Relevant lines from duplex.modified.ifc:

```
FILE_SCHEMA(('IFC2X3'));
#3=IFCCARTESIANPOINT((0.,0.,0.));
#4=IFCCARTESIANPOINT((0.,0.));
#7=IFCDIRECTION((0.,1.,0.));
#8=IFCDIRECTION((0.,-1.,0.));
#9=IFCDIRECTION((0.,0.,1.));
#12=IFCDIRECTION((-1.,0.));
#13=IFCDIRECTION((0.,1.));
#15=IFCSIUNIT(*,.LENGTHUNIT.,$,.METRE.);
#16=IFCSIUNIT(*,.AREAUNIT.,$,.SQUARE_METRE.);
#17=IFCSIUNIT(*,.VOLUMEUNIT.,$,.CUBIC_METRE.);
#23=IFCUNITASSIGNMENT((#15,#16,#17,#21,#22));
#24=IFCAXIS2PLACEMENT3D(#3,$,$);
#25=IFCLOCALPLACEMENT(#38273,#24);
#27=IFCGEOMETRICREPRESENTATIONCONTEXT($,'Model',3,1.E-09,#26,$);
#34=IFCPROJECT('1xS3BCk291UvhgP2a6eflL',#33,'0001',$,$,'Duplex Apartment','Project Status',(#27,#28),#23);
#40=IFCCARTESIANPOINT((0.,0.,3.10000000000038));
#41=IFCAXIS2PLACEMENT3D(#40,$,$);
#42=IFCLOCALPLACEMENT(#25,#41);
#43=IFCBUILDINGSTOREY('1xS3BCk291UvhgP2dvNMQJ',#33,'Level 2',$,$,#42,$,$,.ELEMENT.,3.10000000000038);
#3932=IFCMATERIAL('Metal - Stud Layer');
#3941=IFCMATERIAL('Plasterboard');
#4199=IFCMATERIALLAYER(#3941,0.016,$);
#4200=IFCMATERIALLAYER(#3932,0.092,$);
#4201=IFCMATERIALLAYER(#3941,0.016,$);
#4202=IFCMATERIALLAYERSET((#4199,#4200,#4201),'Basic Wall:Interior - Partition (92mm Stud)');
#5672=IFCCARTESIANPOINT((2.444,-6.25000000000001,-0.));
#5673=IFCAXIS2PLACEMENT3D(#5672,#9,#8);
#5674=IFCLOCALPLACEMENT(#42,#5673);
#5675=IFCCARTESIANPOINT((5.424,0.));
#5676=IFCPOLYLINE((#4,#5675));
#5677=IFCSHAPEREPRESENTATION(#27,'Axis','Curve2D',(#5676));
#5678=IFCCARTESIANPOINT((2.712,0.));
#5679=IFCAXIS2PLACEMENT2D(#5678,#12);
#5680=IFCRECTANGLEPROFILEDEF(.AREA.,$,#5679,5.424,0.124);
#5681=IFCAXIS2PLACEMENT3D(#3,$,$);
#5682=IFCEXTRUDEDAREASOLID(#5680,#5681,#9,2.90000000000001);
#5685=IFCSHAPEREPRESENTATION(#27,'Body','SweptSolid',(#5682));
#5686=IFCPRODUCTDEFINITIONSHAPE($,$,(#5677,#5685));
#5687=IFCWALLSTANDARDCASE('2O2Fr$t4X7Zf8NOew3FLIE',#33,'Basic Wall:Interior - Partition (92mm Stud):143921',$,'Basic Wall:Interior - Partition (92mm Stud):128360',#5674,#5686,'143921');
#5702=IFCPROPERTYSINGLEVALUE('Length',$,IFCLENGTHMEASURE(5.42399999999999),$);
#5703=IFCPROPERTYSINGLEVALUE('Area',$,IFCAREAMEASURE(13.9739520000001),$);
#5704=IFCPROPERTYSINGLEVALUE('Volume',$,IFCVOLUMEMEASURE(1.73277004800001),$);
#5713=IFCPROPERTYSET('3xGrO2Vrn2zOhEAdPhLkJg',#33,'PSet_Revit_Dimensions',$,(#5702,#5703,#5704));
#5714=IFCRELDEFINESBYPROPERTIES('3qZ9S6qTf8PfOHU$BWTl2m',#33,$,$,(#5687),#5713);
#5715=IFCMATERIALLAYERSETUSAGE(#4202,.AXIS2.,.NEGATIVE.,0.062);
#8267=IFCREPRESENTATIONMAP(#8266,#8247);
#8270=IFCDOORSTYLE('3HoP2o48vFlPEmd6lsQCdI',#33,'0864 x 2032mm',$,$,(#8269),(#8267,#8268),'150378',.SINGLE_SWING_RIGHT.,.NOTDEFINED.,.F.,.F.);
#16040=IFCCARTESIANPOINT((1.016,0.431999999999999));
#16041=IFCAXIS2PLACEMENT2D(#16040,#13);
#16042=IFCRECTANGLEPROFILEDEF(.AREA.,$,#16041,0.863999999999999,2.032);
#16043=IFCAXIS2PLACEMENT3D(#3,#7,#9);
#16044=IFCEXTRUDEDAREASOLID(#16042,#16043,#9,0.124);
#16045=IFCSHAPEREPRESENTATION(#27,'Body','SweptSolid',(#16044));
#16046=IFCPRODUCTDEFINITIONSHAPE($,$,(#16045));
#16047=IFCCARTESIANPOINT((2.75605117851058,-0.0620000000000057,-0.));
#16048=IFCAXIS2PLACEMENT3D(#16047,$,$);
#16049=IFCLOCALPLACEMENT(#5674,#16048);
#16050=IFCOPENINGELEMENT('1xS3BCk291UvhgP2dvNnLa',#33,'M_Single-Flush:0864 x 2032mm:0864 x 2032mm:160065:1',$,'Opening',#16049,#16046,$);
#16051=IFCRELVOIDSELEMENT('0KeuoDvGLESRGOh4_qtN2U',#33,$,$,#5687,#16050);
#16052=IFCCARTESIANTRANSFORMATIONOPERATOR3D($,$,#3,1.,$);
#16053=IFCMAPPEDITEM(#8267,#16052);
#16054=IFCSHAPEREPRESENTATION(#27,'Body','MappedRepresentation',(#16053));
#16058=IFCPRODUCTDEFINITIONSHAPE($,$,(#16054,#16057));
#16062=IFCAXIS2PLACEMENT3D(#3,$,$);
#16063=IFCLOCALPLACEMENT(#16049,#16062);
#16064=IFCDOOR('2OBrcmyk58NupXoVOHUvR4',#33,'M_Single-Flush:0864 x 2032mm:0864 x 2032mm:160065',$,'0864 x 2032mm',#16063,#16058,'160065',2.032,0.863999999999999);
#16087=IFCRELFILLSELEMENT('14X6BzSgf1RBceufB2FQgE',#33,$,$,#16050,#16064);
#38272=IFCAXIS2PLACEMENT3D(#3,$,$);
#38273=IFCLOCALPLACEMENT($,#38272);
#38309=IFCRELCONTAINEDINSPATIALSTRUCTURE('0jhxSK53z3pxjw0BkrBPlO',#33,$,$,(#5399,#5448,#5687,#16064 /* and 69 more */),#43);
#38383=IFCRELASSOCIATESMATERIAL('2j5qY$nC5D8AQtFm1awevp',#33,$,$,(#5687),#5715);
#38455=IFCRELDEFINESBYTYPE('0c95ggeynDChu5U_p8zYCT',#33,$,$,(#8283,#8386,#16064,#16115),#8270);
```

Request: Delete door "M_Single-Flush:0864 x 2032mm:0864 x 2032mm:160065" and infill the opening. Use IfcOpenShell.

```python
import ifcopenshell
import ifcopenshell.api.feature
import ifcopenshell.api.pset
import ifcopenshell.api.root
import ifcopenshell.geom
import ifcopenshell.util.element
import ifcopenshell.util.shape
import ifcopenshell.util.unit

model = ifcopenshell.open("duplex.modified.ifc")
area_scale = ifcopenshell.util.unit.calculate_unit_scale(model, "AREAUNIT")
volume_scale = ifcopenshell.util.unit.calculate_unit_scale(model, "VOLUMEUNIT")
settings = ifcopenshell.geom.settings()


def volume(element):
    """Net volume in cubic metres, openings subtracted."""
    shape = ifcopenshell.geom.create_shape(settings, element)
    return ifcopenshell.util.shape.get_volume(shape.geometry)


door = model.by_id(16064)
opening = door.FillsVoids[0].RelatingOpeningElement
wall = opening.VoidsElements[0].RelatingBuildingElement
before = volume(wall)

ifcopenshell.api.root.remove_product(model, product=door)
ifcopenshell.api.feature.remove_feature(model, feature=opening)

after = volume(wall)
thickness = 0.124  # wall thickness in metres

# Update the wall's stored quantities.
pset = model.by_id(ifcopenshell.util.element.get_pset(wall, "PSet_Revit_Dimensions", should_inherit=False)["id"])
ifcopenshell.api.pset.edit_pset(model, pset=pset, properties={
    "Area": model.create_entity("IfcAreaMeasure", after / thickness / area_scale),
    "Volume": model.create_entity("IfcVolumeMeasure", after / volume_scale),
})

print(f"wall volume {before:.3f} -> {after:.3f} m3")

model.write("duplex.modified_rev.ifc")
```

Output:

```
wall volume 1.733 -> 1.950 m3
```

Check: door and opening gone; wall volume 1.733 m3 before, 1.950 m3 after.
